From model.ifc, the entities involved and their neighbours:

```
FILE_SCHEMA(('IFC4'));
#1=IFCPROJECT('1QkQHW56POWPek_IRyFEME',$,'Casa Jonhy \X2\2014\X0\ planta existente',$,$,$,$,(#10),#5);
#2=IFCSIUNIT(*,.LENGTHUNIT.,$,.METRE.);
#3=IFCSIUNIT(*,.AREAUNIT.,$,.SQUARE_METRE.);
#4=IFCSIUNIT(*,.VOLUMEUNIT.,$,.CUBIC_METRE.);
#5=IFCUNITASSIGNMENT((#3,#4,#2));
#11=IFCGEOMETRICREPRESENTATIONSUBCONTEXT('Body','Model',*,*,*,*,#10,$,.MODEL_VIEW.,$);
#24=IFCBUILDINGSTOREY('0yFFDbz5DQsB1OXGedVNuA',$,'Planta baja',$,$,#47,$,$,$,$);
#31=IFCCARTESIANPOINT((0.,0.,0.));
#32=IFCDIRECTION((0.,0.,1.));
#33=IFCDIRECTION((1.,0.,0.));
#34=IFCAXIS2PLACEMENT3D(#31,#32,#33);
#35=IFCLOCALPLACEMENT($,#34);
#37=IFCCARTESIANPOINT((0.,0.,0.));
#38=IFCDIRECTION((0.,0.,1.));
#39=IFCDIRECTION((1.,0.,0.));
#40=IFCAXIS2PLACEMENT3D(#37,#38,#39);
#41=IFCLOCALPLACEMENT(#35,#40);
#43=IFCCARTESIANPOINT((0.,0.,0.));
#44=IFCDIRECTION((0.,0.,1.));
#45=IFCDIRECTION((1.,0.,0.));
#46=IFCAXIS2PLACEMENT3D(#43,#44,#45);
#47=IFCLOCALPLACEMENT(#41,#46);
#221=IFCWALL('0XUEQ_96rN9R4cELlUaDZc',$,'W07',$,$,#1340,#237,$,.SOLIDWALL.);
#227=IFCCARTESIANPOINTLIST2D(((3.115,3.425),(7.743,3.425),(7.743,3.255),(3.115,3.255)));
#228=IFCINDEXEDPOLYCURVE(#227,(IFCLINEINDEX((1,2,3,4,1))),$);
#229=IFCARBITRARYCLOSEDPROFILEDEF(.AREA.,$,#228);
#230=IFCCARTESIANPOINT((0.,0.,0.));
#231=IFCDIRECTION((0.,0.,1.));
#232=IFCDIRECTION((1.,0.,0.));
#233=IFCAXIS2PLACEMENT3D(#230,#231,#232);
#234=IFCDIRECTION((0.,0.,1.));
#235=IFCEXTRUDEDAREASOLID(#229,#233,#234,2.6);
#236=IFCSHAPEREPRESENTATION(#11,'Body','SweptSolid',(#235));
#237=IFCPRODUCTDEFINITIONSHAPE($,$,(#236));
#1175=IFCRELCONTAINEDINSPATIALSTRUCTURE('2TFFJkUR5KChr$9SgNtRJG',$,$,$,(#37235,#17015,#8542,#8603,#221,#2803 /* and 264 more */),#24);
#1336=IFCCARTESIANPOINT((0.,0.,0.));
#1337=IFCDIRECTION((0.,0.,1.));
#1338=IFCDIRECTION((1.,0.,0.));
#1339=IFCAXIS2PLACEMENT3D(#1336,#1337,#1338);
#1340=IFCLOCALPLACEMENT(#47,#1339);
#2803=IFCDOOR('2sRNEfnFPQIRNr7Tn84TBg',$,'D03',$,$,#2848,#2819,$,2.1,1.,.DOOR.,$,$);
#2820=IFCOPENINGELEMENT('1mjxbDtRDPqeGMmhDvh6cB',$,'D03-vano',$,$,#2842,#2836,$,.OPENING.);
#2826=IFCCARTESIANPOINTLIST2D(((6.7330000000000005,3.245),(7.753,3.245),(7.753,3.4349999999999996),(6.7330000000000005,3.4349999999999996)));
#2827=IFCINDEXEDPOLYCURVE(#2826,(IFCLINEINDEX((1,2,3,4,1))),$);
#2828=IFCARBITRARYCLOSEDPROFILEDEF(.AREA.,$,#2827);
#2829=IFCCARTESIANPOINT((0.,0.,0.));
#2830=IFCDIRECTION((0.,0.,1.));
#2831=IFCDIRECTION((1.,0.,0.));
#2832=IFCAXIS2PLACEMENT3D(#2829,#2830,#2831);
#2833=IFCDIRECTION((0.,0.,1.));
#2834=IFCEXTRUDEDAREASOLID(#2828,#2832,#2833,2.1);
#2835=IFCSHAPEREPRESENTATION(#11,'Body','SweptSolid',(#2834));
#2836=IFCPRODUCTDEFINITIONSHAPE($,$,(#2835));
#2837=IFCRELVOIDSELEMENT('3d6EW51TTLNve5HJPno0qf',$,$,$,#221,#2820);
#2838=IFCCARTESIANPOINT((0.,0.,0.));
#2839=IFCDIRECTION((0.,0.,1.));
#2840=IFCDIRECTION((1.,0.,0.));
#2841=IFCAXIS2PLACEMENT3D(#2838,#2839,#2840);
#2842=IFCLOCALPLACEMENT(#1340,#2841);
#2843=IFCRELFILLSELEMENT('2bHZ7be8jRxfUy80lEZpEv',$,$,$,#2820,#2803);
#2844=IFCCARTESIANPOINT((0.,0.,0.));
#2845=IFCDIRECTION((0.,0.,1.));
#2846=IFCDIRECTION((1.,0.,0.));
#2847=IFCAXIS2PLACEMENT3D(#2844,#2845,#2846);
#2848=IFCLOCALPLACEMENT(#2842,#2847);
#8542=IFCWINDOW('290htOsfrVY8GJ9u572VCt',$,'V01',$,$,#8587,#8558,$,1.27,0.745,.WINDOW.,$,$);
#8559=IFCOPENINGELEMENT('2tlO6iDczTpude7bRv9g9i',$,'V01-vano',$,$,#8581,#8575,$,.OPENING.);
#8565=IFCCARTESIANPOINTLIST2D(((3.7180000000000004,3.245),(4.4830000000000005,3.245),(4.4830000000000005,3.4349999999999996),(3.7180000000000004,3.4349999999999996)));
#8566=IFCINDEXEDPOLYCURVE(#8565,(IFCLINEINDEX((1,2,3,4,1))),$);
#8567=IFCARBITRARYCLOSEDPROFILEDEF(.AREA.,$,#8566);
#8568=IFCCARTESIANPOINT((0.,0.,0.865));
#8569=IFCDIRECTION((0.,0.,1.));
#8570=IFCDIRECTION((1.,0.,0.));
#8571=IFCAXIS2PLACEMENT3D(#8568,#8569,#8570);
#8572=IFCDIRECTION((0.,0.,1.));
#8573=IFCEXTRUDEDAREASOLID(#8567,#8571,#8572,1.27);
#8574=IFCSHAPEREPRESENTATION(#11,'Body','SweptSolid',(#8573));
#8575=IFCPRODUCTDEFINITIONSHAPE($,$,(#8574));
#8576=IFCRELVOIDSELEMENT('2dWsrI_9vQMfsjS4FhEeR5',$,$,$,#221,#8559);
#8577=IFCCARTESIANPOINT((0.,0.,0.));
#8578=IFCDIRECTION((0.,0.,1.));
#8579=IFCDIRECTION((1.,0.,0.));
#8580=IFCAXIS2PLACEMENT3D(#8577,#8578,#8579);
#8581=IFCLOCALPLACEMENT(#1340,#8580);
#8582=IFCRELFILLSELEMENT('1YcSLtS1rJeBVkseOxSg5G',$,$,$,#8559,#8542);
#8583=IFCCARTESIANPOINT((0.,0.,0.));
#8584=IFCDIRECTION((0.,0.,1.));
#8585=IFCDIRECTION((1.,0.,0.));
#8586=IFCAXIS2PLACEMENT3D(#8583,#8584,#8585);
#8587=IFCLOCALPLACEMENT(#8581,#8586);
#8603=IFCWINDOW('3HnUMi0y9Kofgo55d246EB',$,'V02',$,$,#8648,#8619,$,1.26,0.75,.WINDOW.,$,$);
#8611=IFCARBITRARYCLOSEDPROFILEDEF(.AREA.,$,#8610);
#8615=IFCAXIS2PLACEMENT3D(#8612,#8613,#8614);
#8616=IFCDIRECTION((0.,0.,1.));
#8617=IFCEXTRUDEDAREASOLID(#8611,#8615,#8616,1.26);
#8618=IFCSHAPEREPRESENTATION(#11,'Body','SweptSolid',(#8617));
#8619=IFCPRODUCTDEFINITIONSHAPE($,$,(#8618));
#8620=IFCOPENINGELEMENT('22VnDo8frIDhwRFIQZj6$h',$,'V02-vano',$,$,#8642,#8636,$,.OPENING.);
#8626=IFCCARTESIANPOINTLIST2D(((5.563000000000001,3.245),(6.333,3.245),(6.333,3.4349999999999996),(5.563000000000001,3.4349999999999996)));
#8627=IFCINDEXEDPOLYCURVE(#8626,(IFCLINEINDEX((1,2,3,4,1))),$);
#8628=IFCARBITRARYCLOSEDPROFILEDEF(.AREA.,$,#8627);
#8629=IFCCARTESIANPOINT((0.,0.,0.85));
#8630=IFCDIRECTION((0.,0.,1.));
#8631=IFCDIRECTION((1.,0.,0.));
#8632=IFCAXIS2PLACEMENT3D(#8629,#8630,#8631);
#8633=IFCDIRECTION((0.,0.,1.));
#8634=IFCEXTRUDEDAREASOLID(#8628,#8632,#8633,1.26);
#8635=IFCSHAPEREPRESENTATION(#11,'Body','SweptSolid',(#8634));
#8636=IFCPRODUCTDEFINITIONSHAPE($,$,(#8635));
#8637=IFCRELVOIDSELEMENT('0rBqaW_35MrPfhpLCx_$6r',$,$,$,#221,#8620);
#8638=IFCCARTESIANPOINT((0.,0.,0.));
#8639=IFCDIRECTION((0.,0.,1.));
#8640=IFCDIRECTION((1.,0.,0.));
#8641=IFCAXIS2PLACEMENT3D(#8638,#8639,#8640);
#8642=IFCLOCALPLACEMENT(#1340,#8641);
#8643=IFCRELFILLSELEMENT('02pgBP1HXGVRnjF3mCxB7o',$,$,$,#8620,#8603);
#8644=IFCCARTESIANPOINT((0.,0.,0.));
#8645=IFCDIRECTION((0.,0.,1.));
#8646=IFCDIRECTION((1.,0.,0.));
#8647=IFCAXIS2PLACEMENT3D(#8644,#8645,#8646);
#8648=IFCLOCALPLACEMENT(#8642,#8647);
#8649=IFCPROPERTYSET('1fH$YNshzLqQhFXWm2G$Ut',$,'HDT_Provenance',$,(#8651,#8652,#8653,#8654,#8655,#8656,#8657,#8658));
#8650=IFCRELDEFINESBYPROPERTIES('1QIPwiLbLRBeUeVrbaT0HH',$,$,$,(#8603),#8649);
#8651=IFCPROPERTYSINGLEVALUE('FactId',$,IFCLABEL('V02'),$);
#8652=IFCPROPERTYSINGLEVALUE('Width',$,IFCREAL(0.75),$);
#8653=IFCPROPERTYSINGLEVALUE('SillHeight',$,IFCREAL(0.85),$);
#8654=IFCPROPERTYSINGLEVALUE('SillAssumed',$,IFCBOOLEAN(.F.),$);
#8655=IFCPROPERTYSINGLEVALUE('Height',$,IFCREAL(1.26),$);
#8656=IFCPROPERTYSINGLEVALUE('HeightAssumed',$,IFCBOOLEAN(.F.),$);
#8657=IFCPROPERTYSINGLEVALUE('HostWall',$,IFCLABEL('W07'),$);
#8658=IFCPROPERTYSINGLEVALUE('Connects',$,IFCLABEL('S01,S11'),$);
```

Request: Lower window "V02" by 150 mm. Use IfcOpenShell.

```python
import numpy as np
import ifcopenshell
import ifcopenshell.api.geometry
import ifcopenshell.api.pset
import ifcopenshell.util.element
import ifcopenshell.util.placement
import ifcopenshell.util.unit

model = ifcopenshell.open("model.ifc")
unit_scale = ifcopenshell.util.unit.calculate_unit_scale(model)

window = model.by_id(8603)
opening = window.FillsVoids[0].RelatingOpeningElement
dz = -0.15 / unit_scale

shift = np.array([0.0, 0.0, dz])
# The window is placed relative to its opening, so it follows when the opening moves.
matrix = ifcopenshell.util.placement.get_local_placement(opening.ObjectPlacement)
matrix[:3, 3] += shift
ifcopenshell.api.geometry.edit_object_placement(
    model, product=opening, matrix=matrix, is_si=False, should_transform_children=True
)

# Keep the stored heights in step.
pset = model.by_id(ifcopenshell.util.element.get_pset(window, "HDT_Provenance", should_inherit=False)["id"])
ifcopenshell.api.pset.edit_pset(model, pset=pset, properties={
    "SillHeight": model.create_entity("IfcReal", ifcopenshell.util.element.get_pset(window, "HDT_Provenance", "SillHeight") + dz),
})

print(f"moved by {dz * unit_scale:+.3f} m")

model.write("model_v2.ifc")
```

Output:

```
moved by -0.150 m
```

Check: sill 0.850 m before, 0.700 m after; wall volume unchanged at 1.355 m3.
